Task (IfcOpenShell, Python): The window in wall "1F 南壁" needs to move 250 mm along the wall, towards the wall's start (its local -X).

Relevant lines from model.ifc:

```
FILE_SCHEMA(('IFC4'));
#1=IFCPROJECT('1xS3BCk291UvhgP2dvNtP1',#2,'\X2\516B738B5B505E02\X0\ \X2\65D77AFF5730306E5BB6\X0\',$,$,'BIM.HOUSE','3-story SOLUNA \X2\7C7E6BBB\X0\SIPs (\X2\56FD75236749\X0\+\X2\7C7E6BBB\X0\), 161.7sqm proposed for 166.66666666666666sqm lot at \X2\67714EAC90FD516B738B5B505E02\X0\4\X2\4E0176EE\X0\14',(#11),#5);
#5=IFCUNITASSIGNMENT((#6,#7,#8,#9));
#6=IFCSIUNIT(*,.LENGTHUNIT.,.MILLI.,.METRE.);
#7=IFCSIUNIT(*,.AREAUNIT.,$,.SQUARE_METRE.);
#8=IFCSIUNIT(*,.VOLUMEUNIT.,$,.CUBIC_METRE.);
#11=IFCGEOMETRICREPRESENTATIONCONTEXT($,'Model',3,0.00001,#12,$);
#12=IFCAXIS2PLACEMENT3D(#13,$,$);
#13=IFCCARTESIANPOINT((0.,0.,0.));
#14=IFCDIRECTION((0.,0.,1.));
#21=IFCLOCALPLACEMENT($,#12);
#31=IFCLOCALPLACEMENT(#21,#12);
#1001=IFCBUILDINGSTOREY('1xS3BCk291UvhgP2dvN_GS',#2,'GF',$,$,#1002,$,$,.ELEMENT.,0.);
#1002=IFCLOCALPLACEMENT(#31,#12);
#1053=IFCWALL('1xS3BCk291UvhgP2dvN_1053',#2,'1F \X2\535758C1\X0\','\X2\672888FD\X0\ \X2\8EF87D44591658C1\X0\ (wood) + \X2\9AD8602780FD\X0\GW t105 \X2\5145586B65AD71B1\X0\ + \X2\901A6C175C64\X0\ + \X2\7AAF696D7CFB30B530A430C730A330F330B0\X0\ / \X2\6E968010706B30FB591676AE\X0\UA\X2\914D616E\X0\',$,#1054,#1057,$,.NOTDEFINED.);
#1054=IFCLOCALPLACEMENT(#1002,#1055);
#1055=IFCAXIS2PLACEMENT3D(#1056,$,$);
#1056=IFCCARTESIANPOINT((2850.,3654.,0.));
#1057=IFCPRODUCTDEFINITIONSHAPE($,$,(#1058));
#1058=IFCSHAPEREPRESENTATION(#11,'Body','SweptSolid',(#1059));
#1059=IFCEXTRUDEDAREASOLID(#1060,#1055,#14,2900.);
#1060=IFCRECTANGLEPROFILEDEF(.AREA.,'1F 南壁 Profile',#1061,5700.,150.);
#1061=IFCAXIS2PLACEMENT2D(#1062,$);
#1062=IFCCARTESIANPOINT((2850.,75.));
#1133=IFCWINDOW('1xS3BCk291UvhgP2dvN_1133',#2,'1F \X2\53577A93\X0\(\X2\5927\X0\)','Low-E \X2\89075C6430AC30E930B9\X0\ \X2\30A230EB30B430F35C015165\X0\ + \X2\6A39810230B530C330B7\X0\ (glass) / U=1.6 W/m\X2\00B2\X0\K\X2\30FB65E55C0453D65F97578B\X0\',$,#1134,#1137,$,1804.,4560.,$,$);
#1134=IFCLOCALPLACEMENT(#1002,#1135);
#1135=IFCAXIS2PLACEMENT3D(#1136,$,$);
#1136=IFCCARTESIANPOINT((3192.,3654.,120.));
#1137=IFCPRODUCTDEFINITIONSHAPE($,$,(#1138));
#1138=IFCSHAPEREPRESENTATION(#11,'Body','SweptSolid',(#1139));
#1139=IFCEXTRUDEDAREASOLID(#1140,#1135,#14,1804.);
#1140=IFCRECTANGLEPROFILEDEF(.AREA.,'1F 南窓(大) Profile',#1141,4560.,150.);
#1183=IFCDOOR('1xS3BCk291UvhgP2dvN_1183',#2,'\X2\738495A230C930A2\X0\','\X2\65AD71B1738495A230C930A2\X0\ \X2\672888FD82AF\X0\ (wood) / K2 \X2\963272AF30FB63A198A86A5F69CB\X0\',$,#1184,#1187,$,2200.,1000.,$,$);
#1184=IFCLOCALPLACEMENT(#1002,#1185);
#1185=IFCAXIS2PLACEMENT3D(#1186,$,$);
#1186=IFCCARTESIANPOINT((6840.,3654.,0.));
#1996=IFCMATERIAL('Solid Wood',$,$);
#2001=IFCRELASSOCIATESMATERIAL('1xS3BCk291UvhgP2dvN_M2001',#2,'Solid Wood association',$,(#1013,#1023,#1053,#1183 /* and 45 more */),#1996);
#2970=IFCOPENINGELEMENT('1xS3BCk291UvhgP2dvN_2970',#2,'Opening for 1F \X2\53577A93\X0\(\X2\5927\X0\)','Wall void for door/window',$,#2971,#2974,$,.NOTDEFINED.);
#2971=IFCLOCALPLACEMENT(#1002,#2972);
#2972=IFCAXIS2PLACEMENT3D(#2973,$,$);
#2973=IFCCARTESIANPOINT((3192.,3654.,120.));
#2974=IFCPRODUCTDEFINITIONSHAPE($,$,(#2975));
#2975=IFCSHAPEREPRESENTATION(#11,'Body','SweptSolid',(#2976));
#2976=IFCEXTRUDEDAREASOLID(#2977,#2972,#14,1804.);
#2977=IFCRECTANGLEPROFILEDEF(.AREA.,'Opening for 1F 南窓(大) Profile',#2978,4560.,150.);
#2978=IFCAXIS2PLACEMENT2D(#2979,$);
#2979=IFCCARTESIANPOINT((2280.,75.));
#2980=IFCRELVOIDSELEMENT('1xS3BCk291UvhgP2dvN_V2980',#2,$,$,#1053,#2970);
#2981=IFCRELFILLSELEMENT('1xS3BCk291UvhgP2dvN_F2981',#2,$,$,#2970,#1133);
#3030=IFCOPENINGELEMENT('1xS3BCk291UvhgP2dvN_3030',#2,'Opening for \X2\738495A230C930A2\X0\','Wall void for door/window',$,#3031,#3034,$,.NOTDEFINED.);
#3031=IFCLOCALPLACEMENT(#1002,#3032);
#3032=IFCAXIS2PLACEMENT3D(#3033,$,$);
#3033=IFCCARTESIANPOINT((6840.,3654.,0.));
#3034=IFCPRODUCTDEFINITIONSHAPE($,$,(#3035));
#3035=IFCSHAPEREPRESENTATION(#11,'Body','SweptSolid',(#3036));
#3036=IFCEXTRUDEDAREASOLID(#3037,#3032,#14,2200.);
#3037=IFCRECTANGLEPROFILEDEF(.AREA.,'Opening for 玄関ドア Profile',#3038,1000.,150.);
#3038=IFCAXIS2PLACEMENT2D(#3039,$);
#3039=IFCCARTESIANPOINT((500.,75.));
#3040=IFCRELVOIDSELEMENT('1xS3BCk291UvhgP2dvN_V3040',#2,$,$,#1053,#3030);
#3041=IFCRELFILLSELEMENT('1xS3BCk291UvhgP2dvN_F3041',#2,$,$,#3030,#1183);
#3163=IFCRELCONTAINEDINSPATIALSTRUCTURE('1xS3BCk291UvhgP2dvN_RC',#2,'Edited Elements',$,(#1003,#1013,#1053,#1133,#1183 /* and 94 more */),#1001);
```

```python
import ifcopenshell
import ifcopenshell.api.geometry
import ifcopenshell.util.placement
import ifcopenshell.util.unit

model = ifcopenshell.open("model.ifc")
unit_scale = ifcopenshell.util.unit.calculate_unit_scale(model)

window = model.by_guid("1xS3BCk291UvhgP2dvN_1133")
opening = window.FillsVoids[0].RelatingOpeningElement
wall = opening.VoidsElements[0].RelatingBuildingElement

wall_matrix = ifcopenshell.util.placement.get_local_placement(wall.ObjectPlacement)
shift = wall_matrix[:3, 0] * -0.25 / unit_scale
before = ifcopenshell.util.placement.get_local_placement(window.ObjectPlacement)[:3, 3].copy()

# The window is not placed relative to its opening, so move both.
for product in (opening, window):
    matrix = ifcopenshell.util.placement.get_local_placement(product.ObjectPlacement)
    matrix[:3, 3] += shift
    ifcopenshell.api.geometry.edit_object_placement(model, product=product, matrix=matrix, is_si=False)

after = ifcopenshell.util.placement.get_local_placement(window.ObjectPlacement)[:3, 3]
print("window moved by", (after - before).round(3) + 0.0)

model.write("model_edited.ifc")
```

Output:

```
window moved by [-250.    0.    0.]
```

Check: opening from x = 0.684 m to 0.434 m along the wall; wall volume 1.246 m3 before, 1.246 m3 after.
